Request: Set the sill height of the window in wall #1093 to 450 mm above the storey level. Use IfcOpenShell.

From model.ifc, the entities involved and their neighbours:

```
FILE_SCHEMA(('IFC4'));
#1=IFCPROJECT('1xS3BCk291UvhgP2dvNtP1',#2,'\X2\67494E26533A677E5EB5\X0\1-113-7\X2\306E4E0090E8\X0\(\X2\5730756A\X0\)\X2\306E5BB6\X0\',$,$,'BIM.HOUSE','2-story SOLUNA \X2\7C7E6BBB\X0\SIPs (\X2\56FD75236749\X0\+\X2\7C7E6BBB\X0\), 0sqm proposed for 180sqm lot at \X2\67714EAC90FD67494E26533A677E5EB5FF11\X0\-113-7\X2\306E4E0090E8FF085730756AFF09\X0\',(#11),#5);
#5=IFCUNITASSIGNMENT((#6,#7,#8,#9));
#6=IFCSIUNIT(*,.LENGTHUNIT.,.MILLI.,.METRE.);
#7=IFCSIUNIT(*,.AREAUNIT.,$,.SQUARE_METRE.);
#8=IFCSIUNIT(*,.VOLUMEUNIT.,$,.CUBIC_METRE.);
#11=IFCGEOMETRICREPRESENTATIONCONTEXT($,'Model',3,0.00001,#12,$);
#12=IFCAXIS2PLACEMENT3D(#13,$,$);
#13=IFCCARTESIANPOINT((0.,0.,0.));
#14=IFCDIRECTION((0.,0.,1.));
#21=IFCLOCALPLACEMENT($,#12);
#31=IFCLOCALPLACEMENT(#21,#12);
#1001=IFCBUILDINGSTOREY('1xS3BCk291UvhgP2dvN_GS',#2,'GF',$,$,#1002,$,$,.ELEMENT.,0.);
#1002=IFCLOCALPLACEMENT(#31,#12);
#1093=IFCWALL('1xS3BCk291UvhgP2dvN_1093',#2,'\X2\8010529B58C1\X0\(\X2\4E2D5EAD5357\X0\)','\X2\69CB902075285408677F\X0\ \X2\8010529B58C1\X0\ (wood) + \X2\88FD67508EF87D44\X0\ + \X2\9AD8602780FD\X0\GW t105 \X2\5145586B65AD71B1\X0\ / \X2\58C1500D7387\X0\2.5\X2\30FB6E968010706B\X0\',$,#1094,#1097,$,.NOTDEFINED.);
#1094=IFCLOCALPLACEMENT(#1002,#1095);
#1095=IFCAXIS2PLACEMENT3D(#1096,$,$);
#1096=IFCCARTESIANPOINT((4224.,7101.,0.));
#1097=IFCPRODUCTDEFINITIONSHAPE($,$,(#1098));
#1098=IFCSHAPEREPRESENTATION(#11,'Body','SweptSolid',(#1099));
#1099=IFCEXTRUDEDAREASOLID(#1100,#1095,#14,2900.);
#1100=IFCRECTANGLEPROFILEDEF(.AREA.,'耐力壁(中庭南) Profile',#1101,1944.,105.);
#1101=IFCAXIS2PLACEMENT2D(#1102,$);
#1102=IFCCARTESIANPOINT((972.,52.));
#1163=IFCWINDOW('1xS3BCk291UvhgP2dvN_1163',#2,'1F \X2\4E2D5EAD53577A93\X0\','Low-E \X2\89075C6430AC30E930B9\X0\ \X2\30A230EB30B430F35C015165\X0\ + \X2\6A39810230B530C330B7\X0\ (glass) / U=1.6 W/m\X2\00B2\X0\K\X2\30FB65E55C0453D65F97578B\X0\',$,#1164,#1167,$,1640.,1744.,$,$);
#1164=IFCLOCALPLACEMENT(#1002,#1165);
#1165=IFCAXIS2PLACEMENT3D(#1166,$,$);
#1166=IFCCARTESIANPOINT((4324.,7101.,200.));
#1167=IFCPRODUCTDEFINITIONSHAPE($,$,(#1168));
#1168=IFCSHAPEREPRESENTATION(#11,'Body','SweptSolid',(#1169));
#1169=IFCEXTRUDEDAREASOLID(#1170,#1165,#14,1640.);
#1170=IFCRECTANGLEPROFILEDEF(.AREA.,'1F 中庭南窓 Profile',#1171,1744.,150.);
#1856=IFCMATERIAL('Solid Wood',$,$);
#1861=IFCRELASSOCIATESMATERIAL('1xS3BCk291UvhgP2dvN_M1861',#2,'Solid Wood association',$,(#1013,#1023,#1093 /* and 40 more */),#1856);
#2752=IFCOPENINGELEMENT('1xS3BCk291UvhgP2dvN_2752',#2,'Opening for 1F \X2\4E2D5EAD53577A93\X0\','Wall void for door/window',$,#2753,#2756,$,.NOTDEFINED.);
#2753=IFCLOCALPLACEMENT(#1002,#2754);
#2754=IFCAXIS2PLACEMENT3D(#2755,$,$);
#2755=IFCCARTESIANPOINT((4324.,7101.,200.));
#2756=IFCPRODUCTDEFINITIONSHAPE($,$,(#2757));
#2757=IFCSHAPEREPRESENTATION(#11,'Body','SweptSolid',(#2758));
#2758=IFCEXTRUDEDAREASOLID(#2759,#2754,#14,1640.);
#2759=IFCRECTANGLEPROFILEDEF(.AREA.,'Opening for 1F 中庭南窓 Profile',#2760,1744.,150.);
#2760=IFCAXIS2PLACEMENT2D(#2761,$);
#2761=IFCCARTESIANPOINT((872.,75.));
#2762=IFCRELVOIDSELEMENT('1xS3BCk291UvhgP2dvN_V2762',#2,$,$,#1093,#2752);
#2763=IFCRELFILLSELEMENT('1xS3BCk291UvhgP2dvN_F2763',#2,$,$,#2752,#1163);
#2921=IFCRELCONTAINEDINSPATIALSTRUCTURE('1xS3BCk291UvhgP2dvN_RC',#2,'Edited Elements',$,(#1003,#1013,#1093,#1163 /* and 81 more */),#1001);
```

```python
import numpy as np
import ifcopenshell
import ifcopenshell.api.geometry
import ifcopenshell.geom
import ifcopenshell.util.element
import ifcopenshell.util.placement
import ifcopenshell.util.shape
import ifcopenshell.util.unit

model = ifcopenshell.open("model.ifc")
unit_scale = ifcopenshell.util.unit.calculate_unit_scale(model)

window = model.by_guid("1xS3BCk291UvhgP2dvN_1163")
opening = window.FillsVoids[0].RelatingOpeningElement
storey = ifcopenshell.util.element.get_container(window, ifc_class="IfcBuildingStorey")
level = ifcopenshell.util.placement.get_local_placement(storey.ObjectPlacement)[2, 3]

# The opening's origin need not be at the sill, so measure its lowest point.
shape = ifcopenshell.geom.create_shape(ifcopenshell.geom.settings(), opening)
bottom = ifcopenshell.util.shape.get_shape_bottom_elevation(shape, shape.geometry) / unit_scale
dz = level + 0.45 / unit_scale - bottom

shift = np.array([0.0, 0.0, dz])
# The window is not placed relative to its opening, so move both.
for product in (opening, window):
    matrix = ifcopenshell.util.placement.get_local_placement(product.ObjectPlacement)
    matrix[:3, 3] += shift
    ifcopenshell.api.geometry.edit_object_placement(model, product=product, matrix=matrix, is_si=False)

print(f"moved by {dz * unit_scale:+.3f} m")

model.write("model_updated.ifc")
```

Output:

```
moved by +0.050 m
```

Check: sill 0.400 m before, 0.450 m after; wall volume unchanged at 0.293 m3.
